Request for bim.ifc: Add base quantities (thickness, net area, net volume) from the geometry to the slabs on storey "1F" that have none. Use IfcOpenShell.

First a look at what the model holds.

```python
import ifcopenshell
import ifcopenshell.util.element
import ifcopenshell.util.unit

model = ifcopenshell.open("bim.ifc")
print(model.schema)
for unit_type in ("LENGTHUNIT", "AREAUNIT", "VOLUMEUNIT"):
    print(unit_type, ifcopenshell.util.unit.calculate_unit_scale(model, unit_type))
storey = next(s for s in model.by_type("IfcBuildingStorey") if s.Name == "1F")
slabs = [e for e in ifcopenshell.util.element.get_decomposition(storey) if e.is_a("IfcSlab")]
for e in sorted(slabs, key=lambda e: e.id()):
    print(e.id(), e.is_a(), e.Name, list(ifcopenshell.util.element.get_psets(e, qtos_only=True)), sep=" | ")
```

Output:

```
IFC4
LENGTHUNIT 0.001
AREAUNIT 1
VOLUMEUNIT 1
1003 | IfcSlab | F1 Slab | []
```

```python
import ifcopenshell
import ifcopenshell.api.pset
import ifcopenshell.geom
import ifcopenshell.util.element
import ifcopenshell.util.shape
import ifcopenshell.util.unit

model = ifcopenshell.open("bim.ifc")
unit_scale = ifcopenshell.util.unit.calculate_unit_scale(model)
area_scale = ifcopenshell.util.unit.calculate_unit_scale(model, "AREAUNIT")
volume_scale = ifcopenshell.util.unit.calculate_unit_scale(model, "VOLUMEUNIT")
settings = ifcopenshell.geom.settings()

storey = next(s for s in model.by_type("IfcBuildingStorey") if s.Name == "1F")
slabs = [e for e in ifcopenshell.util.element.get_decomposition(storey) if e.is_a("IfcSlab")]

for e in sorted(slabs, key=lambda e: e.id()):
    if ifcopenshell.util.element.get_psets(e, qtos_only=True, should_inherit=False):
        continue
    # Geometry comes back in metres, in the element's own axes.
    shape = ifcopenshell.geom.create_shape(settings, e)
    values = {
        "Width": ifcopenshell.util.shape.get_z(shape.geometry) / unit_scale,
        "NetArea": ifcopenshell.util.shape.get_footprint_area(shape.geometry) / area_scale,
        "NetVolume": ifcopenshell.util.shape.get_volume(shape.geometry) / volume_scale,
    }
    qto = ifcopenshell.api.pset.add_qto(model, product=e, name="Qto_SlabBaseQuantities")
    ifcopenshell.api.pset.edit_qto(model, qto=qto, properties=values)
    print(e.id(), {k: round(v, 3) for k, v in values.items()})

model.write("bim_rev.ifc")
```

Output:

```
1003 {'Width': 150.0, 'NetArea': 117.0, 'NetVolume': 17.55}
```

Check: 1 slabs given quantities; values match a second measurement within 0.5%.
